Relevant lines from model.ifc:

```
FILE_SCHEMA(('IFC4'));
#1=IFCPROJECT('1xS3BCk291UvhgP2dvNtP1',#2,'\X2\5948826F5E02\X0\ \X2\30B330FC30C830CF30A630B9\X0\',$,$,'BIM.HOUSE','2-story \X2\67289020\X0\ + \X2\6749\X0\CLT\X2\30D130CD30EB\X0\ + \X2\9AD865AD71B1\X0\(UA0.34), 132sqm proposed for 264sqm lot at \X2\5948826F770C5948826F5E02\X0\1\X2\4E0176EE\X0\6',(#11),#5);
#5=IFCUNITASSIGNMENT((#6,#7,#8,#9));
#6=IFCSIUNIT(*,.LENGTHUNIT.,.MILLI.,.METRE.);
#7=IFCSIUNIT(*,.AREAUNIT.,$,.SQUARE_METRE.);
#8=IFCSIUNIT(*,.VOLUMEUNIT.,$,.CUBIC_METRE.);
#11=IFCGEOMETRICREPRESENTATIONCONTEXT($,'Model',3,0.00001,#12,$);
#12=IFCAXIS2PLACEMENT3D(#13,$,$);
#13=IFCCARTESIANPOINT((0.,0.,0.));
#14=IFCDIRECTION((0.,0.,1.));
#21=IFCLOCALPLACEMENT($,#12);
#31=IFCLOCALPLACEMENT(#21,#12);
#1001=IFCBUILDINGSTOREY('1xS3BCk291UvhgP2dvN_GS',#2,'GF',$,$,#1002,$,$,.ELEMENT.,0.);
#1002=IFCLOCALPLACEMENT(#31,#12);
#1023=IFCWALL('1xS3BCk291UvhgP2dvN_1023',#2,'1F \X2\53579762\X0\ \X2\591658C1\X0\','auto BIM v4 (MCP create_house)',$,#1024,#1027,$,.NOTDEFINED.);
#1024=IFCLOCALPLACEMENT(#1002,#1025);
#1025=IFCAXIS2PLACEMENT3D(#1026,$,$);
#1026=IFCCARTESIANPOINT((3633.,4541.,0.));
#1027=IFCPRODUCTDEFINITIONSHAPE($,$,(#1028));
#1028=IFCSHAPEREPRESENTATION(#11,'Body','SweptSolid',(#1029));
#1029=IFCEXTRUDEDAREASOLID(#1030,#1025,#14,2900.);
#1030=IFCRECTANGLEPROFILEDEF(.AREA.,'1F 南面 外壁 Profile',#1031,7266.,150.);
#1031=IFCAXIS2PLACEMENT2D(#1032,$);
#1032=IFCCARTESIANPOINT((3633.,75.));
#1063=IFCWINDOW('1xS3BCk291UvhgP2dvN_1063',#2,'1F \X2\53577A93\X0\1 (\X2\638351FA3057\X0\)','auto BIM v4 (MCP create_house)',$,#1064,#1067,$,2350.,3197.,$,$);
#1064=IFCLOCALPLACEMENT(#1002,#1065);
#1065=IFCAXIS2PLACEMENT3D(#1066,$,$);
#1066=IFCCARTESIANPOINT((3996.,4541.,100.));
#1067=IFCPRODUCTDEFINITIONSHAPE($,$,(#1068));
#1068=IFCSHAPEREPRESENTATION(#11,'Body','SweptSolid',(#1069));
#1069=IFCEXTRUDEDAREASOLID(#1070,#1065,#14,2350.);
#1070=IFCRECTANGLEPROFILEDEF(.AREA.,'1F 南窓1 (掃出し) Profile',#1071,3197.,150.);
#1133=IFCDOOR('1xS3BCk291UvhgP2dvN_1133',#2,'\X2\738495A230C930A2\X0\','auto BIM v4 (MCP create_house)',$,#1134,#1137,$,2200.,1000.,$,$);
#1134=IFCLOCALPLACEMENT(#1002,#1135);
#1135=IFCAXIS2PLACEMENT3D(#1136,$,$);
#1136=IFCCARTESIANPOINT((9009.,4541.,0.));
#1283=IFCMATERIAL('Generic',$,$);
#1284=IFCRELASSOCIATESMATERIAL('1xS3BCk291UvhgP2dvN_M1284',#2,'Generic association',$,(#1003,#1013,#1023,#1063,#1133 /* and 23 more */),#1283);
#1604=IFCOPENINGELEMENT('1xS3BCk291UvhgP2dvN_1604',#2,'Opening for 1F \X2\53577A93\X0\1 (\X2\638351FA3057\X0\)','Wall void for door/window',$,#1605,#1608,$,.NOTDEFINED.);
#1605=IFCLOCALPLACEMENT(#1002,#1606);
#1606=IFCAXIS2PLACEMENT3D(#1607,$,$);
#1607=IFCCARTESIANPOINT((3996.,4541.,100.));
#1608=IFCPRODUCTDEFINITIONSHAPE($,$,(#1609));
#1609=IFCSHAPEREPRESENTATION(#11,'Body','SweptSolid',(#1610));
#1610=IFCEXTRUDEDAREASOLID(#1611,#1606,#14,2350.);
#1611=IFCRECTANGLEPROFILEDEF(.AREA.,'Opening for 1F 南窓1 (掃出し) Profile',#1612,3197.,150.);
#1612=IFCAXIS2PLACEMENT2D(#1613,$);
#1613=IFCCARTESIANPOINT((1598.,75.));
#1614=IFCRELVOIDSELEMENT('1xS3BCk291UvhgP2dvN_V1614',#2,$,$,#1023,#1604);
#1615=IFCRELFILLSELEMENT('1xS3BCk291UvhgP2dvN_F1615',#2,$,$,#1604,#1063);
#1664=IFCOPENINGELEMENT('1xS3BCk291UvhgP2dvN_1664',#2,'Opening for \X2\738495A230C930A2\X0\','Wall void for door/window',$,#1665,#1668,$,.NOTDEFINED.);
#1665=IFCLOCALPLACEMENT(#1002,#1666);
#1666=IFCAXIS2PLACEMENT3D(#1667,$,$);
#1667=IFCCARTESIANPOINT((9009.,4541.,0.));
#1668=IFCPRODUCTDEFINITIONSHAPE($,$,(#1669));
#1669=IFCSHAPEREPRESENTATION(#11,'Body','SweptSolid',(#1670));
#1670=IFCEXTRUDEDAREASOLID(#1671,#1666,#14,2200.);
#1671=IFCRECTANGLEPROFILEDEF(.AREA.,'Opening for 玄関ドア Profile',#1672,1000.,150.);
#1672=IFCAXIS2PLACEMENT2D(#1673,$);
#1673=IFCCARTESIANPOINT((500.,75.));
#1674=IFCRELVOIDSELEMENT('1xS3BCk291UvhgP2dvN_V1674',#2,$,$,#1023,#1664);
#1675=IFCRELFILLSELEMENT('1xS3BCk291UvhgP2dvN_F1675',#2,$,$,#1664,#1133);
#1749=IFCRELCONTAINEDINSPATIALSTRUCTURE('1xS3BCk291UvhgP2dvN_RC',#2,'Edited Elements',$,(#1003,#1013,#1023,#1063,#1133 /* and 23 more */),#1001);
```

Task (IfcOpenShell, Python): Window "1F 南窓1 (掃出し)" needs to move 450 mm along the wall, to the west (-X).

```python
import ifcopenshell
import ifcopenshell.api.geometry
import ifcopenshell.util.placement
import ifcopenshell.util.unit

model = ifcopenshell.open("model.ifc")
unit_scale = ifcopenshell.util.unit.calculate_unit_scale(model)

window = model.by_guid("1xS3BCk291UvhgP2dvN_1063")
opening = window.FillsVoids[0].RelatingOpeningElement
wall = opening.VoidsElements[0].RelatingBuildingElement

wall_matrix = ifcopenshell.util.placement.get_local_placement(wall.ObjectPlacement)
shift = wall_matrix[:3, 0] * -0.45 / unit_scale
before = ifcopenshell.util.placement.get_local_placement(window.ObjectPlacement)[:3, 3].copy()

# The window is not placed relative to its opening, so move both.
for product in (opening, window):
    matrix = ifcopenshell.util.placement.get_local_placement(product.ObjectPlacement)
    matrix[:3, 3] += shift
    ifcopenshell.api.geometry.edit_object_placement(model, product=product, matrix=matrix, is_si=False)

after = ifcopenshell.util.placement.get_local_placement(window.ObjectPlacement)[:3, 3]
print("window moved by", (after - before).round(3) + 0.0)

model.write("model_rev.ifc")
```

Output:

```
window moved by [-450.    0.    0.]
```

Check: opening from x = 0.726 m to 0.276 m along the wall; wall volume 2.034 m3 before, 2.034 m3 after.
